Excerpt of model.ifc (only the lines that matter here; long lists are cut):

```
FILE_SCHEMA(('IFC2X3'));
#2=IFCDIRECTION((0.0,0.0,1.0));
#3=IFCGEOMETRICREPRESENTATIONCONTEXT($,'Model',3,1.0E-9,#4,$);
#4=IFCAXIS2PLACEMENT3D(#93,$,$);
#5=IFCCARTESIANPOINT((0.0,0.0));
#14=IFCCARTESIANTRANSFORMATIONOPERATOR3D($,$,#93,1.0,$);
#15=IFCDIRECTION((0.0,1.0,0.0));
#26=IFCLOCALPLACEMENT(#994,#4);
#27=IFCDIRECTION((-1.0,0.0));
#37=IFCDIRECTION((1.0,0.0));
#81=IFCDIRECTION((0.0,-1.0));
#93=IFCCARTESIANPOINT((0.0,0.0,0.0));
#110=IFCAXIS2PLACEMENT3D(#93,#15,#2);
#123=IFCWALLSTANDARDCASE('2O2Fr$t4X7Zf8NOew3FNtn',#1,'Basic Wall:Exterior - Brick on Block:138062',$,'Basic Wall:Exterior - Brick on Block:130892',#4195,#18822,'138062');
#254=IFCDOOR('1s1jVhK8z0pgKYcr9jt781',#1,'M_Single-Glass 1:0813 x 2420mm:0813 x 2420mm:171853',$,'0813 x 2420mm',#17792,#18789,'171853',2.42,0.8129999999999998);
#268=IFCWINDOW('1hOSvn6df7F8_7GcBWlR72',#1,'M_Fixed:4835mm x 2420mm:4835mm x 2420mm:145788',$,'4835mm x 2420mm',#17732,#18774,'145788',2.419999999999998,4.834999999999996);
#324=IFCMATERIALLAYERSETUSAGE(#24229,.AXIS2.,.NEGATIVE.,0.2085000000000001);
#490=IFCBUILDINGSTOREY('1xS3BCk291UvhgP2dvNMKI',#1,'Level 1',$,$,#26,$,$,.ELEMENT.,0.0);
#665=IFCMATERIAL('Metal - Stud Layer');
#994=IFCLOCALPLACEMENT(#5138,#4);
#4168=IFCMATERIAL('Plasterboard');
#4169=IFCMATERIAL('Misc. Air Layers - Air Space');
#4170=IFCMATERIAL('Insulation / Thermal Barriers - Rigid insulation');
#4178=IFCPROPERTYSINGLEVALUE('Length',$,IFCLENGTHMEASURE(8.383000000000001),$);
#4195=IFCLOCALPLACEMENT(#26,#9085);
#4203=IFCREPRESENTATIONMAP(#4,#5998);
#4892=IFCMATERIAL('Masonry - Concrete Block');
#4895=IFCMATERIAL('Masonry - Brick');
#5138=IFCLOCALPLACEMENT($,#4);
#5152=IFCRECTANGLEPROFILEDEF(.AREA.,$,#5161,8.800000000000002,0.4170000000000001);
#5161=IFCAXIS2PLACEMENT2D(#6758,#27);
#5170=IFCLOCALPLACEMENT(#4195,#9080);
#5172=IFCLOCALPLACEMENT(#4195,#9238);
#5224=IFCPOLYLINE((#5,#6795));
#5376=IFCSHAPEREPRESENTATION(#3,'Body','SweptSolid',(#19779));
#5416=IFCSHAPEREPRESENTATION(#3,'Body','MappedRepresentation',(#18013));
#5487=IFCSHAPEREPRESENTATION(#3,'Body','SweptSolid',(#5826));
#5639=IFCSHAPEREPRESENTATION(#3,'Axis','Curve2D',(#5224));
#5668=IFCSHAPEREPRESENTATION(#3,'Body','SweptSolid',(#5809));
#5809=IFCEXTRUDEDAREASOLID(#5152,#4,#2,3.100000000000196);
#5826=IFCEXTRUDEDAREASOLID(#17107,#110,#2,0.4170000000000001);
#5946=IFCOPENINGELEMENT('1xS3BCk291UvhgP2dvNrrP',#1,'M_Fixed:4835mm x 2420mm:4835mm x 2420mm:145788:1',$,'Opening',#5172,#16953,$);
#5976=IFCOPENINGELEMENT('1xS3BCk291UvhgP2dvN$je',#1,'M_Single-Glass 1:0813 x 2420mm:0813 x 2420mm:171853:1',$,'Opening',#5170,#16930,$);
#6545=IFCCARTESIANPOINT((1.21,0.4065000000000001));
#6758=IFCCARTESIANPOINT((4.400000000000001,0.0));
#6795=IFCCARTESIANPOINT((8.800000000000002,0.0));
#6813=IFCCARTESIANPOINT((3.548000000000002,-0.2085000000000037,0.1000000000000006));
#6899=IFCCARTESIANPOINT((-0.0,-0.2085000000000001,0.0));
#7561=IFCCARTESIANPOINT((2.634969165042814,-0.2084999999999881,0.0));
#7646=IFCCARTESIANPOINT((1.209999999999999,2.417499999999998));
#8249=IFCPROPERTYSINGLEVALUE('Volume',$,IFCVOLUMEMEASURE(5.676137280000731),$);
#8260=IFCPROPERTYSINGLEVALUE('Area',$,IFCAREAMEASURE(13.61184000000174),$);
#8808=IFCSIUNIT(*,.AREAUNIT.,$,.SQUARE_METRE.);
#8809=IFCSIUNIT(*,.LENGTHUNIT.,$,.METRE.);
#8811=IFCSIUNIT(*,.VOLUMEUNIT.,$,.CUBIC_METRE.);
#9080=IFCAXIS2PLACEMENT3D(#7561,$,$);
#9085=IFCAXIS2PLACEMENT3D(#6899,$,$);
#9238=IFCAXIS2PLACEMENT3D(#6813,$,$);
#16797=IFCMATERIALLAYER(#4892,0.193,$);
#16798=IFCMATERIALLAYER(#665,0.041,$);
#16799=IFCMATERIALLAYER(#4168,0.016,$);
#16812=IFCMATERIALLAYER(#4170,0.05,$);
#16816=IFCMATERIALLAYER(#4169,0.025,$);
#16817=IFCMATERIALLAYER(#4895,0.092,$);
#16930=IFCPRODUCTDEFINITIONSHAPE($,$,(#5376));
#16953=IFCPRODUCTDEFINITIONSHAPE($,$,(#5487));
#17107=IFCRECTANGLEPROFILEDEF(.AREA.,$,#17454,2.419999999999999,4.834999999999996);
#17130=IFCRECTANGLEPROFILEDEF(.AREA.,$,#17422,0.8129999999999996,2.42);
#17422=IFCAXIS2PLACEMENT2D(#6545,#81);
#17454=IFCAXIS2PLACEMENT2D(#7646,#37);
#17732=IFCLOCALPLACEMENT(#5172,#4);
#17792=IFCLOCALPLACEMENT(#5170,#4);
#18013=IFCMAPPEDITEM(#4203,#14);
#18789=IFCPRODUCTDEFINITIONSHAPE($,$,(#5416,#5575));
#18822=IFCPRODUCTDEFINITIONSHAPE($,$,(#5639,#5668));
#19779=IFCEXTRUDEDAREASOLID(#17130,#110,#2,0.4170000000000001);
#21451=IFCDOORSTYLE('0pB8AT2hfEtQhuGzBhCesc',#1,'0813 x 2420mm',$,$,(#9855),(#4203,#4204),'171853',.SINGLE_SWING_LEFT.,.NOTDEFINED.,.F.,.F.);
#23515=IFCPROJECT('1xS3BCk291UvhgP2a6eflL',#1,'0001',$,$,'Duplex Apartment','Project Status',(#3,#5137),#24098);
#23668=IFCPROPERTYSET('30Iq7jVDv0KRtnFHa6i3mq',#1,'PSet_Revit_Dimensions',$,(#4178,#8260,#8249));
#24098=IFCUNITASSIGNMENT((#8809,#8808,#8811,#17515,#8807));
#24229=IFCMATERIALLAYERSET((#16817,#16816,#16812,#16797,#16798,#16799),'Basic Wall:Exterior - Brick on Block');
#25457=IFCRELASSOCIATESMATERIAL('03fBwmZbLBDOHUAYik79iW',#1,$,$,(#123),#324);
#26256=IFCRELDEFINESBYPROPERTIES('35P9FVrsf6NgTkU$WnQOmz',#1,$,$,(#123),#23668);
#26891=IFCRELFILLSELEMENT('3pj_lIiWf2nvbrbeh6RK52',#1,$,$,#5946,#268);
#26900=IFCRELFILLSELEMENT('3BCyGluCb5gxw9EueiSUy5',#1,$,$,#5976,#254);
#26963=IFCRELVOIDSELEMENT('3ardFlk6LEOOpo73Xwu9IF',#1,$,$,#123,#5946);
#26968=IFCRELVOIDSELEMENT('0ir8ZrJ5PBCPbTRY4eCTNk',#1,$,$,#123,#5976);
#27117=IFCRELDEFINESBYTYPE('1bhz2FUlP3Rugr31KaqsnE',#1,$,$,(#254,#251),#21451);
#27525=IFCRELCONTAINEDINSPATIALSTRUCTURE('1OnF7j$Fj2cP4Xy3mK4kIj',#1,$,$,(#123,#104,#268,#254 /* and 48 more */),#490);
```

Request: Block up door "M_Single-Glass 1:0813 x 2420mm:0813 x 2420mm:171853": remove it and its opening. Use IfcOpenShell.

```python
import ifcopenshell
import ifcopenshell.api.feature
import ifcopenshell.api.pset
import ifcopenshell.api.root
import ifcopenshell.geom
import ifcopenshell.util.element
import ifcopenshell.util.shape
import ifcopenshell.util.unit

model = ifcopenshell.open("model.ifc")
area_scale = ifcopenshell.util.unit.calculate_unit_scale(model, "AREAUNIT")
volume_scale = ifcopenshell.util.unit.calculate_unit_scale(model, "VOLUMEUNIT")
settings = ifcopenshell.geom.settings()


def volume(element):
    """Net volume in cubic metres, openings subtracted."""
    shape = ifcopenshell.geom.create_shape(settings, element)
    return ifcopenshell.util.shape.get_volume(shape.geometry)


door = model.by_guid("1s1jVhK8z0pgKYcr9jt781")
opening = door.FillsVoids[0].RelatingOpeningElement
wall = opening.VoidsElements[0].RelatingBuildingElement
before = volume(wall)

ifcopenshell.api.root.remove_product(model, product=door)
ifcopenshell.api.feature.remove_feature(model, feature=opening)

after = volume(wall)
thickness = 0.417  # wall thickness in metres

# Update the wall's stored quantities.
pset = model.by_id(ifcopenshell.util.element.get_pset(wall, "PSet_Revit_Dimensions", should_inherit=False)["id"])
ifcopenshell.api.pset.edit_pset(model, pset=pset, properties={
    "Area": model.create_entity("IfcAreaMeasure", after / thickness / area_scale),
    "Volume": model.create_entity("IfcVolumeMeasure", after / volume_scale),
})

print(f"wall volume {before:.3f} -> {after:.3f} m3")

model.write("model_rev.ifc")
```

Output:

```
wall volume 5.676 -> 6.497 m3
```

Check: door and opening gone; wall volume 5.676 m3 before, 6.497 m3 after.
